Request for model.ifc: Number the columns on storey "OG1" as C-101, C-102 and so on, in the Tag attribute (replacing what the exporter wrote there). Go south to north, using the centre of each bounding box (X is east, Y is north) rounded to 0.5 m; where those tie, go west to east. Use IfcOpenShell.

First a look at what the model holds.

```python
import ifcopenshell
import ifcopenshell.util.element
import ifcopenshell.util.placement

model = ifcopenshell.open("model.ifc")
print(model.schema)
storey = next(s for s in model.by_type("IfcBuildingStorey") if s.Name == "OG1")
columns = [e for e in ifcopenshell.util.element.get_decomposition(storey) if e.is_a("IfcColumn")]
for e in sorted(columns, key=lambda e: e.id()):
    origin = ifcopenshell.util.placement.get_local_placement(e.ObjectPlacement)[:3, 3]
    print(e.id(), e.Tag, e.Name, origin.round(2) + 0.0, sep=" | ")
```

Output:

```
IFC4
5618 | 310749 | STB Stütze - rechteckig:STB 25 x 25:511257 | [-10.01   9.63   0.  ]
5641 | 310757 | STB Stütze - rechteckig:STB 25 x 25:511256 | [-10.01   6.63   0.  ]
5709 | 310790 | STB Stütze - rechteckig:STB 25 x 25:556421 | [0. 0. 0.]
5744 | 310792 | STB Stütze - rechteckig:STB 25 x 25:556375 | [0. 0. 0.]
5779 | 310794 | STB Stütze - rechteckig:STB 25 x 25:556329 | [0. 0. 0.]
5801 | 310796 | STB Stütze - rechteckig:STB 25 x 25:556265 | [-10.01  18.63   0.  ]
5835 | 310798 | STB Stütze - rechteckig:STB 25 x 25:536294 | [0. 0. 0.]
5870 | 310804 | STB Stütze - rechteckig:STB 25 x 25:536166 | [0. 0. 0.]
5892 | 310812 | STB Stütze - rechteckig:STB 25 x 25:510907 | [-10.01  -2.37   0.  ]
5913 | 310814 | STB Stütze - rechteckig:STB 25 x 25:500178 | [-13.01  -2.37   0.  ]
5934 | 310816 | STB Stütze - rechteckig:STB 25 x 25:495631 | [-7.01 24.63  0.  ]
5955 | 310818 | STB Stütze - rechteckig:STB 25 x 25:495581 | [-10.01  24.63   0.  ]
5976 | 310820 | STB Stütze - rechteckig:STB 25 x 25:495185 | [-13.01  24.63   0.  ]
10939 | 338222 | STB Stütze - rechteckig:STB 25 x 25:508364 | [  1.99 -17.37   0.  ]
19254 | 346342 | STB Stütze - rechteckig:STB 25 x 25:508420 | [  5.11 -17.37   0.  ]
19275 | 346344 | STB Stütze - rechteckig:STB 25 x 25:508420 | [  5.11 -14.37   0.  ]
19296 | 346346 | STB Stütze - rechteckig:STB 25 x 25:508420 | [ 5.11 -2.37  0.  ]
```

```python
import ifcopenshell
import ifcopenshell.geom
import ifcopenshell.util.element
import ifcopenshell.util.shape

model = ifcopenshell.open("model.ifc")
settings = ifcopenshell.geom.settings()
settings.set("use-world-coords", True)


def centre(element):
    shape = ifcopenshell.geom.create_shape(settings, element)
    return ifcopenshell.util.shape.get_bbox_centroid(shape.geometry)


storey = next(s for s in model.by_type("IfcBuildingStorey") if s.Name == "OG1")
columns = [e for e in ifcopenshell.util.element.get_decomposition(storey) if e.is_a("IfcColumn")]

# Insertion points can sit at a corner or the storey origin, so sort by the geometry (in metres).
centres = {e: centre(e) for e in columns}
columns.sort(key=lambda e: (round(centres[e][1] / 0.5), centres[e][0]))

for i, e in enumerate(columns, start=1):
    number = f"C-1{i:02d}"
    e.Tag = number
    print(e.id(), number)

model.write("model_edited.ifc")
```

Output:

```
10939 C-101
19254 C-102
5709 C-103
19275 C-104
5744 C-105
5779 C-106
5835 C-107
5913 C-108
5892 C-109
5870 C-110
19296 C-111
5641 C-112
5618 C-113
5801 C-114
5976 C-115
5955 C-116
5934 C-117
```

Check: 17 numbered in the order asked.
